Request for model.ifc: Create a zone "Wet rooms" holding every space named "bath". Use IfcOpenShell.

First a look at what the model holds.

```python
import ifcopenshell

model = ifcopenshell.open("model.ifc")
print(model.schema)
seen = {}
for space in model.by_type("IfcSpace"):
    seen[space.LongName] = seen.get(space.LongName, 0) + 1
for name, count in sorted(seen.items(), key=str):
    print(count, "x", name)
print("zones:", [z.Name for z in model.by_type("IfcZone")][:20])
```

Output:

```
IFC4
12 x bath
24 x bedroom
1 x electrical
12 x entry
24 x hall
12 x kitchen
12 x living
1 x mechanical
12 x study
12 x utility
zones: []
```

```python
import ifcopenshell
import ifcopenshell.api.group
import ifcopenshell.api.root

model = ifcopenshell.open("model.ifc")

names = {"bath"}
spaces = [s for s in model.by_type("IfcSpace") if s.LongName in names]

zone = ifcopenshell.api.root.create_entity(model, ifc_class="IfcZone", name="Wet rooms")
ifcopenshell.api.group.assign_group(model, products=spaces, group=zone)
print(len(spaces), "spaces in", zone.Name)

model.write("model_updated.ifc")
```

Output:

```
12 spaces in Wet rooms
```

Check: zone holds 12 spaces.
